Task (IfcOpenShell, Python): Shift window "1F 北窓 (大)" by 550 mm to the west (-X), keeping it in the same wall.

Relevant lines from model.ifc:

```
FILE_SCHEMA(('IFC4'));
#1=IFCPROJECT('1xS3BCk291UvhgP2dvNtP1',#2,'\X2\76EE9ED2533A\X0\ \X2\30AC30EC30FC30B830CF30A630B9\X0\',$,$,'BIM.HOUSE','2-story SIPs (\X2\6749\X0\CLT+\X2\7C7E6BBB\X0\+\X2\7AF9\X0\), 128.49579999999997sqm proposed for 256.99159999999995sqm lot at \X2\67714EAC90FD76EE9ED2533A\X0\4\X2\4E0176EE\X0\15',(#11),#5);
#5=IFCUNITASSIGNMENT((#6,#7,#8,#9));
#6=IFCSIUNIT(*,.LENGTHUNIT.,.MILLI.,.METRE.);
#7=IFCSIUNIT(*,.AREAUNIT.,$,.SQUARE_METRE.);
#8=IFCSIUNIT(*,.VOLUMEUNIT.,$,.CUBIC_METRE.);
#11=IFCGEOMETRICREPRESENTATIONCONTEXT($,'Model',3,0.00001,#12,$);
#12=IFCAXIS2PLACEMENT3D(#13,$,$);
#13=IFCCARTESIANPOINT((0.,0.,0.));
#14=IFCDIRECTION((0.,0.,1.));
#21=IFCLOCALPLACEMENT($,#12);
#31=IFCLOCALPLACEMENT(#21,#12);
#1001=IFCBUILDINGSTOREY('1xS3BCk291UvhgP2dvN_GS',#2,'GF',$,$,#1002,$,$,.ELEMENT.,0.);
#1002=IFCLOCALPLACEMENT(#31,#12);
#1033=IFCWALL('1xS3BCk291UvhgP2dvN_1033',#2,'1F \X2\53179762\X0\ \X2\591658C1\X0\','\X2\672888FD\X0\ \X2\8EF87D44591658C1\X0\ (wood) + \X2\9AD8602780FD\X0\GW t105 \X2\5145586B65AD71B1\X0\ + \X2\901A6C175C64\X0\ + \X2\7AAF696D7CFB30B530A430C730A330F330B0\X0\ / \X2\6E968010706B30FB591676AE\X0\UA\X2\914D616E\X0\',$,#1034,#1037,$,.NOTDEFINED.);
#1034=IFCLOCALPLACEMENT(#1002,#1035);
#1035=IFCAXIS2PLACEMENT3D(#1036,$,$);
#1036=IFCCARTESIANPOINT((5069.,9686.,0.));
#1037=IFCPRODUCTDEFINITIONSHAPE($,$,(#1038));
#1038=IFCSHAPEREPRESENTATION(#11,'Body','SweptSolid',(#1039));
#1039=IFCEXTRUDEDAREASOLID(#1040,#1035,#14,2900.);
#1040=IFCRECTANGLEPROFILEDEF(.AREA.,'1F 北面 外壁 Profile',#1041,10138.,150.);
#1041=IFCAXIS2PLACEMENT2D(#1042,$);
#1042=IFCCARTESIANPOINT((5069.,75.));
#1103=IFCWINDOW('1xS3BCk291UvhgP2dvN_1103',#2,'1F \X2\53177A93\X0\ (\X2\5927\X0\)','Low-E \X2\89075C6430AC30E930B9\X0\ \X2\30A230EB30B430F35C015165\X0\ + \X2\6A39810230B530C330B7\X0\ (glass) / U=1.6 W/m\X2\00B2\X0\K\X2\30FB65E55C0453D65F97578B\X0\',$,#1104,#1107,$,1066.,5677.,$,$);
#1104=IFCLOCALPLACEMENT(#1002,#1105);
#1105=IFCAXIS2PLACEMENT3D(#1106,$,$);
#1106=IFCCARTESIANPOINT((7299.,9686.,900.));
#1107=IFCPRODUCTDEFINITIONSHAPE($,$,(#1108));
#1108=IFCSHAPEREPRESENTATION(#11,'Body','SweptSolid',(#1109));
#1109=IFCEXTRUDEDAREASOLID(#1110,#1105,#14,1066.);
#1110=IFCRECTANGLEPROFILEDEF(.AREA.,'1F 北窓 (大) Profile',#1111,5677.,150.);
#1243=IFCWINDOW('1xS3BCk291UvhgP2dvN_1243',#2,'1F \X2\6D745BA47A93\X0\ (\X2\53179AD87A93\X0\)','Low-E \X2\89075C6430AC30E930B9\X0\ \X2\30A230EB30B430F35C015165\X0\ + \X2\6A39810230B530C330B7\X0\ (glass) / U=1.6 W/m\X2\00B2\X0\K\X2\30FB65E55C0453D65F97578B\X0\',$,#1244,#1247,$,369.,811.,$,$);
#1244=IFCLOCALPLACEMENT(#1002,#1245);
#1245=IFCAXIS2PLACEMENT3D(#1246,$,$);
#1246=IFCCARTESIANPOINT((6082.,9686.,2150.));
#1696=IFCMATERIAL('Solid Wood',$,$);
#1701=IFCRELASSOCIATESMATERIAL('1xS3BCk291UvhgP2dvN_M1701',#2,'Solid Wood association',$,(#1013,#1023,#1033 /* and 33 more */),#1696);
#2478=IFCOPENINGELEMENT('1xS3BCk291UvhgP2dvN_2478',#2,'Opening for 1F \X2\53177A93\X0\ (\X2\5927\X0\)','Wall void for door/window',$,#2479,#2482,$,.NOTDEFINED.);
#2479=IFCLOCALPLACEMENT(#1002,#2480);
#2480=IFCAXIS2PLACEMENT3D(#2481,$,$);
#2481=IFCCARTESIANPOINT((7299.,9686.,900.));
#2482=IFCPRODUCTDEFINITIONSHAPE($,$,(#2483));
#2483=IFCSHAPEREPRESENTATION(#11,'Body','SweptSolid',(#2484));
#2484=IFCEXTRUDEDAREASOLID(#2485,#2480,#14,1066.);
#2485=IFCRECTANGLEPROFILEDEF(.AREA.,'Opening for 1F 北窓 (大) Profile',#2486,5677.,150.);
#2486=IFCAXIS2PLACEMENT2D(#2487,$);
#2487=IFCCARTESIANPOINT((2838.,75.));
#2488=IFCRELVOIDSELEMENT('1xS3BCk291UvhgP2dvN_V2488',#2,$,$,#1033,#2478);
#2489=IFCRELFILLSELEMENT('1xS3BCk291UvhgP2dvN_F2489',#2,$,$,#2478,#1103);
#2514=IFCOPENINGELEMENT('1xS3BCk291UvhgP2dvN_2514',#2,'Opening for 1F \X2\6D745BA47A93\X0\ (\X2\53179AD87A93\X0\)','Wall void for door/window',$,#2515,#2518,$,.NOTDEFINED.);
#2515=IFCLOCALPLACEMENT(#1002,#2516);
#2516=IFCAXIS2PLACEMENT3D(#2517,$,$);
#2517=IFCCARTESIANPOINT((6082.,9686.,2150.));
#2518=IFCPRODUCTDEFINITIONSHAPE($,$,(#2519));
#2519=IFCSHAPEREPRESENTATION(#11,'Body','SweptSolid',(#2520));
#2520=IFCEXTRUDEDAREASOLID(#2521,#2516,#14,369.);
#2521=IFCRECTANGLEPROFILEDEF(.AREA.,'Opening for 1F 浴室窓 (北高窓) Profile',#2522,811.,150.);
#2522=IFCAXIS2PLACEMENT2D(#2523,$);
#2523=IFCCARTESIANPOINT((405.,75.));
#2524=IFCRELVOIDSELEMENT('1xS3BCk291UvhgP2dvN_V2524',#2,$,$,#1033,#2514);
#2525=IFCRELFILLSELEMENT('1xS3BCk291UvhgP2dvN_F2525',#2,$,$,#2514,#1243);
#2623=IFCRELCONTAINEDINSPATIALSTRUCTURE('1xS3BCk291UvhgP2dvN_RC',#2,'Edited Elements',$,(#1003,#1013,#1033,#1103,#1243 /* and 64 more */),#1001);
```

```python
import ifcopenshell
import ifcopenshell.api.geometry
import ifcopenshell.util.placement
import ifcopenshell.util.unit

model = ifcopenshell.open("model.ifc")
unit_scale = ifcopenshell.util.unit.calculate_unit_scale(model)

window = model.by_id(1103)
opening = window.FillsVoids[0].RelatingOpeningElement
wall = opening.VoidsElements[0].RelatingBuildingElement

wall_matrix = ifcopenshell.util.placement.get_local_placement(wall.ObjectPlacement)
shift = wall_matrix[:3, 0] * -0.55 / unit_scale
before = ifcopenshell.util.placement.get_local_placement(window.ObjectPlacement)[:3, 3].copy()

# The window is not placed relative to its opening, so move both.
for product in (opening, window):
    matrix = ifcopenshell.util.placement.get_local_placement(product.ObjectPlacement)
    matrix[:3, 3] += shift
    ifcopenshell.api.geometry.edit_object_placement(model, product=product, matrix=matrix, is_si=False)

after = ifcopenshell.util.placement.get_local_placement(window.ObjectPlacement)[:3, 3]
print("window moved by", (after - before).round(3) + 0.0)

model.write("model_edited.ifc")
```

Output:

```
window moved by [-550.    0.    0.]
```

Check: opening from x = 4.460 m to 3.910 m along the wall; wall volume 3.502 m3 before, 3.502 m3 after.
